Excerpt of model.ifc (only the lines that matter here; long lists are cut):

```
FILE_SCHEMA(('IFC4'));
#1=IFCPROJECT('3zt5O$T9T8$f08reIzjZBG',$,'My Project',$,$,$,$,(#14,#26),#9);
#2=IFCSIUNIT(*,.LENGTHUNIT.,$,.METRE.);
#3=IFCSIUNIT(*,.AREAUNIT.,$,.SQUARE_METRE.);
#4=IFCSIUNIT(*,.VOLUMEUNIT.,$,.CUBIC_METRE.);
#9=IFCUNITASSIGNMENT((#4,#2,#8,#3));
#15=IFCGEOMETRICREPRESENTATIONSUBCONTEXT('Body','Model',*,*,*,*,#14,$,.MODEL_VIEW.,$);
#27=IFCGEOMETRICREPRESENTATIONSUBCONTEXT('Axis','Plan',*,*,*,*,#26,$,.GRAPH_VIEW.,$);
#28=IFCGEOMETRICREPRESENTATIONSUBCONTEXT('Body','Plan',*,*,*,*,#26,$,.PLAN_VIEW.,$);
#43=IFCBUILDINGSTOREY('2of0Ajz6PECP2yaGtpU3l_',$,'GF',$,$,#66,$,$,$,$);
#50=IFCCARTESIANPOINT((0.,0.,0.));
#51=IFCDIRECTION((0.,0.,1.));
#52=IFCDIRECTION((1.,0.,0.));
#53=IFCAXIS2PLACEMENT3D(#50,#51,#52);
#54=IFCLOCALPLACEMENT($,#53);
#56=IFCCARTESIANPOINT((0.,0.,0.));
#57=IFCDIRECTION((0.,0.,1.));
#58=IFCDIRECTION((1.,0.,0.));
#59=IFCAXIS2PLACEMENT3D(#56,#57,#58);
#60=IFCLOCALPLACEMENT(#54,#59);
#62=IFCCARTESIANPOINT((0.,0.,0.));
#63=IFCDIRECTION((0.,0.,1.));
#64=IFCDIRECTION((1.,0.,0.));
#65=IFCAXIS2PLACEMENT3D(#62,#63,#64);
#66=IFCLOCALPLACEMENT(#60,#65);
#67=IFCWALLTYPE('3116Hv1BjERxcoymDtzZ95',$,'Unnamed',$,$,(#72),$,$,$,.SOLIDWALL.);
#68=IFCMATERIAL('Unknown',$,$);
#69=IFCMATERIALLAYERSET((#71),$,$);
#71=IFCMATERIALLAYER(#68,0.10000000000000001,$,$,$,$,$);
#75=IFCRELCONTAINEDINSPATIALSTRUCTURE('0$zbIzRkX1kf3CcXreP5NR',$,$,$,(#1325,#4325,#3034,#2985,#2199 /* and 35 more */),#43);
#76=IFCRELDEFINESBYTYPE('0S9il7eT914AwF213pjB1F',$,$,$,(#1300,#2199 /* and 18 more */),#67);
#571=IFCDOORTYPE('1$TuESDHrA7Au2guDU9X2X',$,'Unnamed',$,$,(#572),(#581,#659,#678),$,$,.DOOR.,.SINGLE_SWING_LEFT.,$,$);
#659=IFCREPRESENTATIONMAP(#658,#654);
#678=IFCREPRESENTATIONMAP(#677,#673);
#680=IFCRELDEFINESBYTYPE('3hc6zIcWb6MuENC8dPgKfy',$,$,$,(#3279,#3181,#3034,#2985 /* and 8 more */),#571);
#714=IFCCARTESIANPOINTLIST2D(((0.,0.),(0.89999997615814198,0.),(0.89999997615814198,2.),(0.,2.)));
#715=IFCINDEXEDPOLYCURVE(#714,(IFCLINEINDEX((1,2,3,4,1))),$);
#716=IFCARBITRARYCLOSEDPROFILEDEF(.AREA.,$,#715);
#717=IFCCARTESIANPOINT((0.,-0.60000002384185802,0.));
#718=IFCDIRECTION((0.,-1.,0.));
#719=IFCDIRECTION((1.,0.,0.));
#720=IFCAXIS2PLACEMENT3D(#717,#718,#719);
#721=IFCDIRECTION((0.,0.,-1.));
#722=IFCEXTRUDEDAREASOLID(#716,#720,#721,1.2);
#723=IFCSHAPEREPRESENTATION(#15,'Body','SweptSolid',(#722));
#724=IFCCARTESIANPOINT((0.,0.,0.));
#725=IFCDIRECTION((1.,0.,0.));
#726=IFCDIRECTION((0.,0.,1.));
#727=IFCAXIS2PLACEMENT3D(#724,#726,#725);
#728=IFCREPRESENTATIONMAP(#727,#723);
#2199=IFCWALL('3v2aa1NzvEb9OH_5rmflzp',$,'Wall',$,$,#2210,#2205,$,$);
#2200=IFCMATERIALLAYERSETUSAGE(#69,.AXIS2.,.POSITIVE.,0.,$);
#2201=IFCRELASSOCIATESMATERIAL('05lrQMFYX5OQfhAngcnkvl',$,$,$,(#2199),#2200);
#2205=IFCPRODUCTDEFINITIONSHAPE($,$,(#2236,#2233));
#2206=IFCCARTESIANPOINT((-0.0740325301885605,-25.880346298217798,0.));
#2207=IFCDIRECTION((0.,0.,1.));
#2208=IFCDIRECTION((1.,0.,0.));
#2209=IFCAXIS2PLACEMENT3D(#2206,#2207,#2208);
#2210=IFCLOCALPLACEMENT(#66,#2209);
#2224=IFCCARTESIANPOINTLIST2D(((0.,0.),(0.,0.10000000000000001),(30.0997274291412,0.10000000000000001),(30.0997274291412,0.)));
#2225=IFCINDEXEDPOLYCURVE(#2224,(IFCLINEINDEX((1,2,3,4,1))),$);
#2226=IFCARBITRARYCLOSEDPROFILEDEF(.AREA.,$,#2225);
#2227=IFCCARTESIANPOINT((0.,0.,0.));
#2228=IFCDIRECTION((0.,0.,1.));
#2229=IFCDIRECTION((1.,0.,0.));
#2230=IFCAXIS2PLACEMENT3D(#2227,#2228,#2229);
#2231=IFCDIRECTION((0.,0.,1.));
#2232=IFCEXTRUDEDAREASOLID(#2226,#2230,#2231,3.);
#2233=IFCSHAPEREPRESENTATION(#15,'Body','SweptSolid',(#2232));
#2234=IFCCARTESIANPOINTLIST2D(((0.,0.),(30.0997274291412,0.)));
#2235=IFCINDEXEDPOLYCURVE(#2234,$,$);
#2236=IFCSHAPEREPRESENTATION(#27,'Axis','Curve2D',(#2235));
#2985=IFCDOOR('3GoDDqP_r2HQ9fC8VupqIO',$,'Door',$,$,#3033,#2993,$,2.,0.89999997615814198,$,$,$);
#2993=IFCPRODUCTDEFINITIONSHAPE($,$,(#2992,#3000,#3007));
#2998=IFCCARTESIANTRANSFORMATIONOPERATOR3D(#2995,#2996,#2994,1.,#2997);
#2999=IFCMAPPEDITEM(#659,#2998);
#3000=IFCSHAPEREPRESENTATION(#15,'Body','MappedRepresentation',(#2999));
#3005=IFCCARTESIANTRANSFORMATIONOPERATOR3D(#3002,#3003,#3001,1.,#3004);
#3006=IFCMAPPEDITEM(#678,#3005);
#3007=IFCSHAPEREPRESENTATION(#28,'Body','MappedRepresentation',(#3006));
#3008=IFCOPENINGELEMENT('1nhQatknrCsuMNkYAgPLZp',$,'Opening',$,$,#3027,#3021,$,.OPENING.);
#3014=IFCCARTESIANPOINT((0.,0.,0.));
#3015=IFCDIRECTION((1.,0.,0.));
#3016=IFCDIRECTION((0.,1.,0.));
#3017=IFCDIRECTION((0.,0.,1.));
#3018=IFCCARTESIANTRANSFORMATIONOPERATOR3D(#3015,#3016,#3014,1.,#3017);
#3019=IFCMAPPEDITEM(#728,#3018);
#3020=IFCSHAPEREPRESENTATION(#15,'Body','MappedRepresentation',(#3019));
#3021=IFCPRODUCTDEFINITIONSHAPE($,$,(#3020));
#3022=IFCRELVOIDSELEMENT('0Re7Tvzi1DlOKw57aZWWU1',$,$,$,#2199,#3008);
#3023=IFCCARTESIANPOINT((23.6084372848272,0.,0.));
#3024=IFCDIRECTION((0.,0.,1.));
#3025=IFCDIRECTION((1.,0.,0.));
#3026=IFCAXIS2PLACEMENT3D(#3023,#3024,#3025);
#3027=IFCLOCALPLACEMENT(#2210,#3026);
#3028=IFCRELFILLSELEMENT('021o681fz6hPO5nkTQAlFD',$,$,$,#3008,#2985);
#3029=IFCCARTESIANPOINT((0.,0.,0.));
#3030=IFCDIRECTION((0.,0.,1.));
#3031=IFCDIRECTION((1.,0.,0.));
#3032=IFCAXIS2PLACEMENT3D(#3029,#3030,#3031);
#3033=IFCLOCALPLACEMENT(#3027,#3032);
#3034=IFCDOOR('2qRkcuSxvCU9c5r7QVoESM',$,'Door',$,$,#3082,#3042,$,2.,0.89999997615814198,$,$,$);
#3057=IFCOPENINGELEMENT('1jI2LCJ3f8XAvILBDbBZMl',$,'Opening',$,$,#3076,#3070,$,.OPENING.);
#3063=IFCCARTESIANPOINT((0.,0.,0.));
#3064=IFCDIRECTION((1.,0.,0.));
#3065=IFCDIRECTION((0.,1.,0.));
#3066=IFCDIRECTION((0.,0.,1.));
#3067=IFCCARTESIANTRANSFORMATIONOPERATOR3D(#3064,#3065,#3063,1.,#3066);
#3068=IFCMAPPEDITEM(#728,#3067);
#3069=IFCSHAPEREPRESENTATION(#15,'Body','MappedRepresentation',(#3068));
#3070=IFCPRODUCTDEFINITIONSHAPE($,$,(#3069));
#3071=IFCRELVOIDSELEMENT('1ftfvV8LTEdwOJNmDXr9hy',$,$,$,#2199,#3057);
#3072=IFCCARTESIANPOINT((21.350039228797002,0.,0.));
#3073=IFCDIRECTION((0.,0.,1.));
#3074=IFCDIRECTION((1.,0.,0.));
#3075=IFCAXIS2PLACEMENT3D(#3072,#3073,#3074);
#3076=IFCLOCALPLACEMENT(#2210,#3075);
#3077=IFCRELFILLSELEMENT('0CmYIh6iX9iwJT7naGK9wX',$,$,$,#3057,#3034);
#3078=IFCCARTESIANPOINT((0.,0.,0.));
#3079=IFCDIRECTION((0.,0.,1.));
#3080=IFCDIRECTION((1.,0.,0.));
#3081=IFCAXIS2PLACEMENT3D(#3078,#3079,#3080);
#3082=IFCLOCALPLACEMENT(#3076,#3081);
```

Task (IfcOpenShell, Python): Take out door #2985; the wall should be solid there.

```python
import ifcopenshell
import ifcopenshell.api.feature
import ifcopenshell.api.root
import ifcopenshell.geom
import ifcopenshell.util.shape

model = ifcopenshell.open("model.ifc")
settings = ifcopenshell.geom.settings()


def volume(element):
    """Net volume in cubic metres, openings subtracted."""
    shape = ifcopenshell.geom.create_shape(settings, element)
    return ifcopenshell.util.shape.get_volume(shape.geometry)


door = model.by_id(2985)
opening = door.FillsVoids[0].RelatingOpeningElement
wall = opening.VoidsElements[0].RelatingBuildingElement
before = volume(wall)

ifcopenshell.api.root.remove_product(model, product=door)
ifcopenshell.api.feature.remove_feature(model, feature=opening)

after = volume(wall)

print(f"wall volume {before:.3f} -> {after:.3f} m3")

model.write("model-out.ifc")
```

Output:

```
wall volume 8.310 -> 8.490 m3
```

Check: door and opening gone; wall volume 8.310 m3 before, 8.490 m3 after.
